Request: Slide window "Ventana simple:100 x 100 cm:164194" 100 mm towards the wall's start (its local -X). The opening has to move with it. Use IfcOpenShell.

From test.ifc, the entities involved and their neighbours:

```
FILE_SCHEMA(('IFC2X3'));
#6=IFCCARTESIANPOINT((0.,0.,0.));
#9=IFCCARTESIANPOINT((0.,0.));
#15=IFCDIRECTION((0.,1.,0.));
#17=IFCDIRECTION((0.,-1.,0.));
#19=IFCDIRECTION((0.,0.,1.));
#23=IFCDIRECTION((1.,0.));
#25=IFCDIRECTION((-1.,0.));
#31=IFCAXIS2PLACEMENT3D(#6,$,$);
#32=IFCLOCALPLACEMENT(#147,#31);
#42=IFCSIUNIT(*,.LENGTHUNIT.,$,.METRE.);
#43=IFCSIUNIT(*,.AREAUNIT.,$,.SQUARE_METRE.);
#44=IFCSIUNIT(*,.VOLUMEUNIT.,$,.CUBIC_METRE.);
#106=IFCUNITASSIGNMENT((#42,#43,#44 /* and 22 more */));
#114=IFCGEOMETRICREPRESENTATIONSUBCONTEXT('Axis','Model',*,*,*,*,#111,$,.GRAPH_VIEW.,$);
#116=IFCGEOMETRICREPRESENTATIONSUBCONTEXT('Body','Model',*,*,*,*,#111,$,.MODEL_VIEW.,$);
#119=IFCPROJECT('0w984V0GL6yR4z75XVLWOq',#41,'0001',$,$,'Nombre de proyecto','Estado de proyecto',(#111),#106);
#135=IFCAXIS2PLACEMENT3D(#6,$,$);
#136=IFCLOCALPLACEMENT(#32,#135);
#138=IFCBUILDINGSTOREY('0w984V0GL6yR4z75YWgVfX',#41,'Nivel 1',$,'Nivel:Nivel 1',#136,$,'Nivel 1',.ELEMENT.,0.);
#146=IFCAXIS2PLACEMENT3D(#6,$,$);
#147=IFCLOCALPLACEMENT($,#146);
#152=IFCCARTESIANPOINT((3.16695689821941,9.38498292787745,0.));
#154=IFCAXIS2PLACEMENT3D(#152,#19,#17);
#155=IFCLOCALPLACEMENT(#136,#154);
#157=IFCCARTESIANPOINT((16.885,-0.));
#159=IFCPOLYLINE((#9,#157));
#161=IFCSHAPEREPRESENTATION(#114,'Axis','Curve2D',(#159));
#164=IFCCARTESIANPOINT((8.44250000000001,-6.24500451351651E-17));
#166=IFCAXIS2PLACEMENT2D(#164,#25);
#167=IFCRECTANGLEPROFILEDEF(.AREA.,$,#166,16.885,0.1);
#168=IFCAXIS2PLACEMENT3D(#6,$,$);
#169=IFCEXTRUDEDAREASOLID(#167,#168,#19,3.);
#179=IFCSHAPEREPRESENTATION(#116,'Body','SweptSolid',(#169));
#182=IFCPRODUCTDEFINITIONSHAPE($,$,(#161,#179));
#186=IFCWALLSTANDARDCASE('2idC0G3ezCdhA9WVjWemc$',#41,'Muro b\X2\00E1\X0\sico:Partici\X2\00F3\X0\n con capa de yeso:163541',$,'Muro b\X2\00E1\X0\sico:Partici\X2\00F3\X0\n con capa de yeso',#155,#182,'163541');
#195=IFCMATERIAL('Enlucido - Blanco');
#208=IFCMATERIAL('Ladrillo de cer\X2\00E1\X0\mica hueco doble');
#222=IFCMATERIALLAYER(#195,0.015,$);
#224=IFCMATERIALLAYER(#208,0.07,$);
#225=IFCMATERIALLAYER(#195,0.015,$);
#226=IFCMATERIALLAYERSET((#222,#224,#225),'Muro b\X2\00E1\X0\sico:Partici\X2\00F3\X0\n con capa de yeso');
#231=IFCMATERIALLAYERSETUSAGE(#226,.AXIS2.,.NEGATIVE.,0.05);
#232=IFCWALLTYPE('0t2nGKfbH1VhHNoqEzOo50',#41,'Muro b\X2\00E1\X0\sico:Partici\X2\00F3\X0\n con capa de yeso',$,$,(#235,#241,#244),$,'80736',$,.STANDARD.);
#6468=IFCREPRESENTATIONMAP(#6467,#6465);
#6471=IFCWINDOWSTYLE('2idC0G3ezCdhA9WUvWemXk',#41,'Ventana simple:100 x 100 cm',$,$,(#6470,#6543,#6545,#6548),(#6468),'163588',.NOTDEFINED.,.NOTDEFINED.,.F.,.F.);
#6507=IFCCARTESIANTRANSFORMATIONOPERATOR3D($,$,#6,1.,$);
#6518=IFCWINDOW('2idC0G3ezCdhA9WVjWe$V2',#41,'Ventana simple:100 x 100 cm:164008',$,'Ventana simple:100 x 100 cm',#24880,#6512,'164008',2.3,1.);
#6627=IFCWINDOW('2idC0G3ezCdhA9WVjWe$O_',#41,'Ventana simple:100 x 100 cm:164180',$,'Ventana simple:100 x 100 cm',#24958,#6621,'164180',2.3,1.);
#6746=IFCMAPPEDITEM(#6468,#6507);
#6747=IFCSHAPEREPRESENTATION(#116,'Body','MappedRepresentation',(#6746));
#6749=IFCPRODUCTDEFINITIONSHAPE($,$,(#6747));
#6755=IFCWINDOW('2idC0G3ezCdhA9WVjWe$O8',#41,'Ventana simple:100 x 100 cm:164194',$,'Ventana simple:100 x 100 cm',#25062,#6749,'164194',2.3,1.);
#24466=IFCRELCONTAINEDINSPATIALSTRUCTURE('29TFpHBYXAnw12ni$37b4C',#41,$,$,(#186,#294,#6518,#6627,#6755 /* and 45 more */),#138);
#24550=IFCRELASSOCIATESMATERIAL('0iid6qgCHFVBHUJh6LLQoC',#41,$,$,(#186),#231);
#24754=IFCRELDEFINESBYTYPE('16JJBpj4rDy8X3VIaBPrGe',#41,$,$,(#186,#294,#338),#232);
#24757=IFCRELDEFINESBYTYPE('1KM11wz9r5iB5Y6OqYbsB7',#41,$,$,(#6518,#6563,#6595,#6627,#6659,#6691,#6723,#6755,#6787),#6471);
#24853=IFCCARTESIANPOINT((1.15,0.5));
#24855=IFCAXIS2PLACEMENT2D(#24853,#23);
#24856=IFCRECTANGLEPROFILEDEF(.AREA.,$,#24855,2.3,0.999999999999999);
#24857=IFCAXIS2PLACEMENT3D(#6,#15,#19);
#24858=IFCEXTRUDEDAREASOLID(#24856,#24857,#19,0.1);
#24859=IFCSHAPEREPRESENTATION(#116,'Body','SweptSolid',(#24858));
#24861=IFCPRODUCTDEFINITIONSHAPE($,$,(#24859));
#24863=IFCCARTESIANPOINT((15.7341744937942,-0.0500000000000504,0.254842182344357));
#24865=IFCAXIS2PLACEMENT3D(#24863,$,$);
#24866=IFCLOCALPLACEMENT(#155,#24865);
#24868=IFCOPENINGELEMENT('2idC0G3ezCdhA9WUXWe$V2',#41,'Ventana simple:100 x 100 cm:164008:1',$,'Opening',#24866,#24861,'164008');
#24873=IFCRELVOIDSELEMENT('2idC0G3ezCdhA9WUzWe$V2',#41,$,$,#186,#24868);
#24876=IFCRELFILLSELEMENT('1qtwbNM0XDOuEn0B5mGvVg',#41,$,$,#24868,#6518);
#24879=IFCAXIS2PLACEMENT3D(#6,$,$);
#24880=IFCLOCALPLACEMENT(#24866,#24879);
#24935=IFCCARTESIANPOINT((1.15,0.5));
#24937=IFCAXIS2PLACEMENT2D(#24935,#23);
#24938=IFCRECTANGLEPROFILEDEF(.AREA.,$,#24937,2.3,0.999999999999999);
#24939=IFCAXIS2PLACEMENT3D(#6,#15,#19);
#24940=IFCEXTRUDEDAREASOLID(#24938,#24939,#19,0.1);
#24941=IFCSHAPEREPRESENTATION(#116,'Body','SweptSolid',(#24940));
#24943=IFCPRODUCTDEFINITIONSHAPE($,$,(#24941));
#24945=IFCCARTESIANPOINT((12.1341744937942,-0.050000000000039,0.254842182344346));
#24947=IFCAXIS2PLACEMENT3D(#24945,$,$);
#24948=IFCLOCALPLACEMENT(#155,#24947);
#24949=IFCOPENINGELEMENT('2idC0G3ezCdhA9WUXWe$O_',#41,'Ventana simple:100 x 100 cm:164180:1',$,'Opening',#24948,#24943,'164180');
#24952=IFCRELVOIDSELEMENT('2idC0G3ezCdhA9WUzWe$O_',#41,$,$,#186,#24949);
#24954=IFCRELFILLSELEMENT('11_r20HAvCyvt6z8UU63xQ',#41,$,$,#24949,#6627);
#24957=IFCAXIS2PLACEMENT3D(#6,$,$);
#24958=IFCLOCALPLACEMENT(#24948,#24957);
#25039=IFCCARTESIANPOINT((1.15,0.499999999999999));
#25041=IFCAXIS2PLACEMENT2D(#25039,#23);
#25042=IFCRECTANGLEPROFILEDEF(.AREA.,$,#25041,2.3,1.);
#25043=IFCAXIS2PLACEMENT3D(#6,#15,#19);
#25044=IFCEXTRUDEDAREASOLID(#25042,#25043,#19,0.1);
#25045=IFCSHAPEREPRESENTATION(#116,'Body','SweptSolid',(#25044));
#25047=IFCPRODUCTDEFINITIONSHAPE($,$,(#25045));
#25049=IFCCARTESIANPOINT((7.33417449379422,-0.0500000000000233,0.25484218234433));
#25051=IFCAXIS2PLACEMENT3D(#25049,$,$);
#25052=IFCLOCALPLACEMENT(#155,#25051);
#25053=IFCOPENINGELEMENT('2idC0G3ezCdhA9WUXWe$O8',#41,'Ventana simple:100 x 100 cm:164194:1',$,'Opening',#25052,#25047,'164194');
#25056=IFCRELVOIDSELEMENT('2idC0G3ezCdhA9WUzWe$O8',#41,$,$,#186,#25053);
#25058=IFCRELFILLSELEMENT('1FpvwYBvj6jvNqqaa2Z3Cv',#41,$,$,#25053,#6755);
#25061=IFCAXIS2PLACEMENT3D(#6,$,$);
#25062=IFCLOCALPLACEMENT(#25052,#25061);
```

```python
import ifcopenshell
import ifcopenshell.api.geometry
import ifcopenshell.util.placement

model = ifcopenshell.open("test.ifc")

window = model.by_guid("2idC0G3ezCdhA9WVjWe$O8")
opening = window.FillsVoids[0].RelatingOpeningElement
wall = opening.VoidsElements[0].RelatingBuildingElement

wall_matrix = ifcopenshell.util.placement.get_local_placement(wall.ObjectPlacement)
shift = wall_matrix[:3, 0] * -0.1
before = ifcopenshell.util.placement.get_local_placement(window.ObjectPlacement)[:3, 3].copy()

# The window is placed relative to its opening, so it follows when the opening moves.
matrix = ifcopenshell.util.placement.get_local_placement(opening.ObjectPlacement)
matrix[:3, 3] += shift
ifcopenshell.api.geometry.edit_object_placement(
    model, product=opening, matrix=matrix, is_si=False, should_transform_children=True
)

after = ifcopenshell.util.placement.get_local_placement(window.ObjectPlacement)[:3, 3]
print("window moved by", (after - before).round(3) + 0.0)

model.write("test_edited.ifc")
```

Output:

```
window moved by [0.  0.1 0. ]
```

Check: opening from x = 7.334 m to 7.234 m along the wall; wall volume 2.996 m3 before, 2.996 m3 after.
